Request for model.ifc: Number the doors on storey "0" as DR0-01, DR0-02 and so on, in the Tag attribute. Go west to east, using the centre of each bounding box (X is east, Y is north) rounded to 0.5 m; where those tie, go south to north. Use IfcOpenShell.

First a look at what the model holds.

```python
import ifcopenshell
import ifcopenshell.util.element
import ifcopenshell.util.placement

model = ifcopenshell.open("model.ifc")
print(model.schema)
storey = next(s for s in model.by_type("IfcBuildingStorey") if s.Name == "0")
doors = [e for e in ifcopenshell.util.element.get_decomposition(storey) if e.is_a("IfcDoor")]
for e in sorted(doors, key=lambda e: e.id()):
    origin = ifcopenshell.util.placement.get_local_placement(e.ObjectPlacement)[:3, 3]
    print(e.id(), e.Tag, e.Name, origin.round(2) + 0.0, sep=" | ")
```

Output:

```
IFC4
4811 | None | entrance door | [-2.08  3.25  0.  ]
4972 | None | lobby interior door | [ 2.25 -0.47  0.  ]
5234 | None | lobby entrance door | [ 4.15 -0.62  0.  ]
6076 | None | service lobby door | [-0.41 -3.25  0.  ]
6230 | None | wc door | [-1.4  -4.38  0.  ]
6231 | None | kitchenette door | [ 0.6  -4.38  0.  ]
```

```python
import ifcopenshell
import ifcopenshell.geom
import ifcopenshell.util.element
import ifcopenshell.util.shape

model = ifcopenshell.open("model.ifc")
settings = ifcopenshell.geom.settings()
settings.set("use-world-coords", True)


def centre(element):
    shape = ifcopenshell.geom.create_shape(settings, element)
    return ifcopenshell.util.shape.get_bbox_centroid(shape.geometry)


storey = next(s for s in model.by_type("IfcBuildingStorey") if s.Name == "0")
doors = [e for e in ifcopenshell.util.element.get_decomposition(storey) if e.is_a("IfcDoor")]

# Insertion points can sit at a corner or the storey origin, so sort by the geometry (in metres).
centres = {e: centre(e) for e in doors}
doors.sort(key=lambda e: (round(centres[e][0] / 0.5), centres[e][1]))

for i, e in enumerate(doors, start=1):
    number = f"DR0-{i:02d}"
    e.Tag = number
    print(e.id(), number)

model.write("model_updated.ifc")
```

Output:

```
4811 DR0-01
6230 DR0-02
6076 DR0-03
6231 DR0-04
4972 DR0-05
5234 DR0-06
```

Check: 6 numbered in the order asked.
